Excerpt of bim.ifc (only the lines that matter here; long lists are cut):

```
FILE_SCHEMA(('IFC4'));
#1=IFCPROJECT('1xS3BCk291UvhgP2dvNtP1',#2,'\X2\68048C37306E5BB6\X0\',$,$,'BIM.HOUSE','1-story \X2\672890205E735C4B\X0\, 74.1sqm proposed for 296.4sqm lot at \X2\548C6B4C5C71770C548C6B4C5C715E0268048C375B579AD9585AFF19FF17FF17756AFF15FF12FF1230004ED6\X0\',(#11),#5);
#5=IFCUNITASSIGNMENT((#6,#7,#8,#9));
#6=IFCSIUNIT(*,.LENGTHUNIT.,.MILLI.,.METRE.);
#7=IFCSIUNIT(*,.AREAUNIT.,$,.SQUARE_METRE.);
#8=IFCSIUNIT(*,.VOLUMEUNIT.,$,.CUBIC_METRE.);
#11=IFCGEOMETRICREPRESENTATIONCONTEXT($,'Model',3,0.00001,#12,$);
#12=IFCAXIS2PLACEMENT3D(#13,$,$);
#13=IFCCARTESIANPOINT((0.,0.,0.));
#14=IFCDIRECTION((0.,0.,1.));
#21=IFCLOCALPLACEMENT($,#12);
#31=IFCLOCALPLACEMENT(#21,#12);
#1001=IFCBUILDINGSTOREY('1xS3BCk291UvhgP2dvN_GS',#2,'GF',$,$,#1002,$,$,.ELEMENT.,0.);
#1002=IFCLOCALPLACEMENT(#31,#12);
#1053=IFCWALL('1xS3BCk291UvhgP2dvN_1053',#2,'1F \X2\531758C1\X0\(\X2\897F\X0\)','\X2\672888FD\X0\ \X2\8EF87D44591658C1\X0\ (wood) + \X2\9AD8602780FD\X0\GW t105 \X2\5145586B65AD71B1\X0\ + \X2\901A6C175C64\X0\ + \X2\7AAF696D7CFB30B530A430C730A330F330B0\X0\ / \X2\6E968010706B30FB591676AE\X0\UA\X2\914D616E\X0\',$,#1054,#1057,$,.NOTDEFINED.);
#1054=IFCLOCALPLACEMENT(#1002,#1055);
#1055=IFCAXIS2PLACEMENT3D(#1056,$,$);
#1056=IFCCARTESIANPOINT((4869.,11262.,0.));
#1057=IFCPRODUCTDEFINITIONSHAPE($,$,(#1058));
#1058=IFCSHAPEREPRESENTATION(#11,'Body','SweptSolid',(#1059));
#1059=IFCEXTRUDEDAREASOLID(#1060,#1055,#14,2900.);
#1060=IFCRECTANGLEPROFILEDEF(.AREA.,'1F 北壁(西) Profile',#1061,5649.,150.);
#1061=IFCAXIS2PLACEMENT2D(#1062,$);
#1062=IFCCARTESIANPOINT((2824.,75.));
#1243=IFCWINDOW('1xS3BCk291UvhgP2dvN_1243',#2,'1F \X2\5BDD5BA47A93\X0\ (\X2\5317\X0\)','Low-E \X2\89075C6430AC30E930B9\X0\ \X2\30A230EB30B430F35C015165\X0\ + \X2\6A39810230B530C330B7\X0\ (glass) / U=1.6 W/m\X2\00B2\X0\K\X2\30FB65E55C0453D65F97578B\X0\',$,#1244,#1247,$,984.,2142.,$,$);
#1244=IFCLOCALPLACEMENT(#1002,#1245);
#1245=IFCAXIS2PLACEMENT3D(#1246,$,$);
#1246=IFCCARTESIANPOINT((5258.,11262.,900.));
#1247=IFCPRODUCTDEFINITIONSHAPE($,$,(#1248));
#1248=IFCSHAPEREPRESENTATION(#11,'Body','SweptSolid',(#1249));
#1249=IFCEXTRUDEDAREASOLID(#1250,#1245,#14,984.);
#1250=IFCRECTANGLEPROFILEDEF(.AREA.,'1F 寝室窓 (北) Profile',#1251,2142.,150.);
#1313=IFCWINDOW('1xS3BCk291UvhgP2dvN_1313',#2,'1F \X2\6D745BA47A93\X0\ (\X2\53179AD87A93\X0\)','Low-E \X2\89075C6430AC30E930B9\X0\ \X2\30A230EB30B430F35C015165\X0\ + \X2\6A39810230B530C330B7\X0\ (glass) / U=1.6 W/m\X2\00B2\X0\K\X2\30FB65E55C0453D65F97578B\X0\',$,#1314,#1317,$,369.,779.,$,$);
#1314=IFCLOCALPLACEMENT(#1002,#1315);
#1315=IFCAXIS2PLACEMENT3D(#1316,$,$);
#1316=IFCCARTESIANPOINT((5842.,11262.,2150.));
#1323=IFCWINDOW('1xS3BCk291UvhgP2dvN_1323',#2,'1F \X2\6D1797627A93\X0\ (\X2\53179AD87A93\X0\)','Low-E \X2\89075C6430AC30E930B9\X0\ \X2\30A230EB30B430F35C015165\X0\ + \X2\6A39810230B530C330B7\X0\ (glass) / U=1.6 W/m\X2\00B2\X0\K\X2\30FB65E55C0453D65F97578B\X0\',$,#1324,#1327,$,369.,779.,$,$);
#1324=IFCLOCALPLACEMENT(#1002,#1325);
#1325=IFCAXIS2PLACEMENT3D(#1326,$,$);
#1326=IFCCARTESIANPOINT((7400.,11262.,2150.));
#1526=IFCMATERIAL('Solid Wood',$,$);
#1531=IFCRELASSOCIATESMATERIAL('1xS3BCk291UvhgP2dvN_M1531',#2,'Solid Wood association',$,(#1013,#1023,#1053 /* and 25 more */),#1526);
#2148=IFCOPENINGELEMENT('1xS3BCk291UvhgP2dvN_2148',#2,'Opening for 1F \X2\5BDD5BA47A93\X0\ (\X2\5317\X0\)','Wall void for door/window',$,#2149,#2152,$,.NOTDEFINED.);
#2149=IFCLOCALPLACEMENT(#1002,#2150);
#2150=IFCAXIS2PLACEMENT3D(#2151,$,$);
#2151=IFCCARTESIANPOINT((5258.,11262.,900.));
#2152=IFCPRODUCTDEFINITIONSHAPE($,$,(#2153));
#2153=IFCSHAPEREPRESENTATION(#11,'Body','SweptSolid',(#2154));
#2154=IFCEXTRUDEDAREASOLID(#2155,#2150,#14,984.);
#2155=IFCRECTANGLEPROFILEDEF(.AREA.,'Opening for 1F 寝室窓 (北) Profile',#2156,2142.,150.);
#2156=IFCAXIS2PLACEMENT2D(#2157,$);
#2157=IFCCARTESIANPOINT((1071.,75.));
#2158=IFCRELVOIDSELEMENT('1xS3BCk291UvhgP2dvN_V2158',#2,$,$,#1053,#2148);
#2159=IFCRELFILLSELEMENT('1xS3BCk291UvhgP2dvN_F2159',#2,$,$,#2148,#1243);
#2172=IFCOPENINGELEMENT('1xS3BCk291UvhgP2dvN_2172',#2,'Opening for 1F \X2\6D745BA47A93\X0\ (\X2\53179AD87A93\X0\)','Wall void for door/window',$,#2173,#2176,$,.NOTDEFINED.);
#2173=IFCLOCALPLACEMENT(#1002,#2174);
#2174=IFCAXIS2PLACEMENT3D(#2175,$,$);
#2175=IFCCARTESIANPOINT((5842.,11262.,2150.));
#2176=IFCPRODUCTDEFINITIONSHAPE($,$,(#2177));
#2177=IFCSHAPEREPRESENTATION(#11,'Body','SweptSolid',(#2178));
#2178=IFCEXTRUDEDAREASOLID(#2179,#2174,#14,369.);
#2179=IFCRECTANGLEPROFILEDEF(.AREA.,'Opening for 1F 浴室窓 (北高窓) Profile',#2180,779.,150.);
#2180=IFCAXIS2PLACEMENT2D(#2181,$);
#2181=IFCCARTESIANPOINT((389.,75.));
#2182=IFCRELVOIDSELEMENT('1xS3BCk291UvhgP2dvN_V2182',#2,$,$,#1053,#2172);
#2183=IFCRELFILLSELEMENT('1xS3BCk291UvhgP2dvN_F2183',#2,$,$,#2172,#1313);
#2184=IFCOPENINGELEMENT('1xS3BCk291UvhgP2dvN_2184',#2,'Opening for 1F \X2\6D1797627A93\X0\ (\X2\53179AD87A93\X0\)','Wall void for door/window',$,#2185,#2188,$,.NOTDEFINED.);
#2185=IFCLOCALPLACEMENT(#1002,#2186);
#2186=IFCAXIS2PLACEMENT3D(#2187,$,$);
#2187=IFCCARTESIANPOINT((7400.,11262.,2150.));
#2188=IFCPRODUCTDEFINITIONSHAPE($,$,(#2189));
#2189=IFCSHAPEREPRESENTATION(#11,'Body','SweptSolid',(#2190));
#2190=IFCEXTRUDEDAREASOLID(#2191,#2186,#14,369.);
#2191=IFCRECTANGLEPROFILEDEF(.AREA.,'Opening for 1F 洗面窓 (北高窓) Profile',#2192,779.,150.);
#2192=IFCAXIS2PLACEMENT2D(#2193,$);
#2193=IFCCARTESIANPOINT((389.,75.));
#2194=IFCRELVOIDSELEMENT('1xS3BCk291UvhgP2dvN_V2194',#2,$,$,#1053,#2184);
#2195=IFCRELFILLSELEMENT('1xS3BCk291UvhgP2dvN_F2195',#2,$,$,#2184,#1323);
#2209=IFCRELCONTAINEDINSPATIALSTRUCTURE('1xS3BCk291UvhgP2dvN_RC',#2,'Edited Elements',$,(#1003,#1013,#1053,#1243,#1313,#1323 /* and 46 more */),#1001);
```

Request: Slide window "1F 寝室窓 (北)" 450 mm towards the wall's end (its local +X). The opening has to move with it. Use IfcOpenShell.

```python
import ifcopenshell
import ifcopenshell.api.geometry
import ifcopenshell.util.placement
import ifcopenshell.util.unit

model = ifcopenshell.open("bim.ifc")
unit_scale = ifcopenshell.util.unit.calculate_unit_scale(model)

window = model.by_id(1243)
opening = window.FillsVoids[0].RelatingOpeningElement
wall = opening.VoidsElements[0].RelatingBuildingElement

wall_matrix = ifcopenshell.util.placement.get_local_placement(wall.ObjectPlacement)
shift = wall_matrix[:3, 0] * 0.45 / unit_scale
before = ifcopenshell.util.placement.get_local_placement(window.ObjectPlacement)[:3, 3].copy()

# The window is not placed relative to its opening, so move both.
for product in (opening, window):
    matrix = ifcopenshell.util.placement.get_local_placement(product.ObjectPlacement)
    matrix[:3, 3] += shift
    ifcopenshell.api.geometry.edit_object_placement(model, product=product, matrix=matrix, is_si=False)

after = ifcopenshell.util.placement.get_local_placement(window.ObjectPlacement)[:3, 3]
print("window moved by", (after - before).round(3) + 0.0)

model.write("bim_edited.ifc")
```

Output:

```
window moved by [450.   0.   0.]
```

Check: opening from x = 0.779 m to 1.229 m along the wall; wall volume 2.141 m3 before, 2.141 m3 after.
